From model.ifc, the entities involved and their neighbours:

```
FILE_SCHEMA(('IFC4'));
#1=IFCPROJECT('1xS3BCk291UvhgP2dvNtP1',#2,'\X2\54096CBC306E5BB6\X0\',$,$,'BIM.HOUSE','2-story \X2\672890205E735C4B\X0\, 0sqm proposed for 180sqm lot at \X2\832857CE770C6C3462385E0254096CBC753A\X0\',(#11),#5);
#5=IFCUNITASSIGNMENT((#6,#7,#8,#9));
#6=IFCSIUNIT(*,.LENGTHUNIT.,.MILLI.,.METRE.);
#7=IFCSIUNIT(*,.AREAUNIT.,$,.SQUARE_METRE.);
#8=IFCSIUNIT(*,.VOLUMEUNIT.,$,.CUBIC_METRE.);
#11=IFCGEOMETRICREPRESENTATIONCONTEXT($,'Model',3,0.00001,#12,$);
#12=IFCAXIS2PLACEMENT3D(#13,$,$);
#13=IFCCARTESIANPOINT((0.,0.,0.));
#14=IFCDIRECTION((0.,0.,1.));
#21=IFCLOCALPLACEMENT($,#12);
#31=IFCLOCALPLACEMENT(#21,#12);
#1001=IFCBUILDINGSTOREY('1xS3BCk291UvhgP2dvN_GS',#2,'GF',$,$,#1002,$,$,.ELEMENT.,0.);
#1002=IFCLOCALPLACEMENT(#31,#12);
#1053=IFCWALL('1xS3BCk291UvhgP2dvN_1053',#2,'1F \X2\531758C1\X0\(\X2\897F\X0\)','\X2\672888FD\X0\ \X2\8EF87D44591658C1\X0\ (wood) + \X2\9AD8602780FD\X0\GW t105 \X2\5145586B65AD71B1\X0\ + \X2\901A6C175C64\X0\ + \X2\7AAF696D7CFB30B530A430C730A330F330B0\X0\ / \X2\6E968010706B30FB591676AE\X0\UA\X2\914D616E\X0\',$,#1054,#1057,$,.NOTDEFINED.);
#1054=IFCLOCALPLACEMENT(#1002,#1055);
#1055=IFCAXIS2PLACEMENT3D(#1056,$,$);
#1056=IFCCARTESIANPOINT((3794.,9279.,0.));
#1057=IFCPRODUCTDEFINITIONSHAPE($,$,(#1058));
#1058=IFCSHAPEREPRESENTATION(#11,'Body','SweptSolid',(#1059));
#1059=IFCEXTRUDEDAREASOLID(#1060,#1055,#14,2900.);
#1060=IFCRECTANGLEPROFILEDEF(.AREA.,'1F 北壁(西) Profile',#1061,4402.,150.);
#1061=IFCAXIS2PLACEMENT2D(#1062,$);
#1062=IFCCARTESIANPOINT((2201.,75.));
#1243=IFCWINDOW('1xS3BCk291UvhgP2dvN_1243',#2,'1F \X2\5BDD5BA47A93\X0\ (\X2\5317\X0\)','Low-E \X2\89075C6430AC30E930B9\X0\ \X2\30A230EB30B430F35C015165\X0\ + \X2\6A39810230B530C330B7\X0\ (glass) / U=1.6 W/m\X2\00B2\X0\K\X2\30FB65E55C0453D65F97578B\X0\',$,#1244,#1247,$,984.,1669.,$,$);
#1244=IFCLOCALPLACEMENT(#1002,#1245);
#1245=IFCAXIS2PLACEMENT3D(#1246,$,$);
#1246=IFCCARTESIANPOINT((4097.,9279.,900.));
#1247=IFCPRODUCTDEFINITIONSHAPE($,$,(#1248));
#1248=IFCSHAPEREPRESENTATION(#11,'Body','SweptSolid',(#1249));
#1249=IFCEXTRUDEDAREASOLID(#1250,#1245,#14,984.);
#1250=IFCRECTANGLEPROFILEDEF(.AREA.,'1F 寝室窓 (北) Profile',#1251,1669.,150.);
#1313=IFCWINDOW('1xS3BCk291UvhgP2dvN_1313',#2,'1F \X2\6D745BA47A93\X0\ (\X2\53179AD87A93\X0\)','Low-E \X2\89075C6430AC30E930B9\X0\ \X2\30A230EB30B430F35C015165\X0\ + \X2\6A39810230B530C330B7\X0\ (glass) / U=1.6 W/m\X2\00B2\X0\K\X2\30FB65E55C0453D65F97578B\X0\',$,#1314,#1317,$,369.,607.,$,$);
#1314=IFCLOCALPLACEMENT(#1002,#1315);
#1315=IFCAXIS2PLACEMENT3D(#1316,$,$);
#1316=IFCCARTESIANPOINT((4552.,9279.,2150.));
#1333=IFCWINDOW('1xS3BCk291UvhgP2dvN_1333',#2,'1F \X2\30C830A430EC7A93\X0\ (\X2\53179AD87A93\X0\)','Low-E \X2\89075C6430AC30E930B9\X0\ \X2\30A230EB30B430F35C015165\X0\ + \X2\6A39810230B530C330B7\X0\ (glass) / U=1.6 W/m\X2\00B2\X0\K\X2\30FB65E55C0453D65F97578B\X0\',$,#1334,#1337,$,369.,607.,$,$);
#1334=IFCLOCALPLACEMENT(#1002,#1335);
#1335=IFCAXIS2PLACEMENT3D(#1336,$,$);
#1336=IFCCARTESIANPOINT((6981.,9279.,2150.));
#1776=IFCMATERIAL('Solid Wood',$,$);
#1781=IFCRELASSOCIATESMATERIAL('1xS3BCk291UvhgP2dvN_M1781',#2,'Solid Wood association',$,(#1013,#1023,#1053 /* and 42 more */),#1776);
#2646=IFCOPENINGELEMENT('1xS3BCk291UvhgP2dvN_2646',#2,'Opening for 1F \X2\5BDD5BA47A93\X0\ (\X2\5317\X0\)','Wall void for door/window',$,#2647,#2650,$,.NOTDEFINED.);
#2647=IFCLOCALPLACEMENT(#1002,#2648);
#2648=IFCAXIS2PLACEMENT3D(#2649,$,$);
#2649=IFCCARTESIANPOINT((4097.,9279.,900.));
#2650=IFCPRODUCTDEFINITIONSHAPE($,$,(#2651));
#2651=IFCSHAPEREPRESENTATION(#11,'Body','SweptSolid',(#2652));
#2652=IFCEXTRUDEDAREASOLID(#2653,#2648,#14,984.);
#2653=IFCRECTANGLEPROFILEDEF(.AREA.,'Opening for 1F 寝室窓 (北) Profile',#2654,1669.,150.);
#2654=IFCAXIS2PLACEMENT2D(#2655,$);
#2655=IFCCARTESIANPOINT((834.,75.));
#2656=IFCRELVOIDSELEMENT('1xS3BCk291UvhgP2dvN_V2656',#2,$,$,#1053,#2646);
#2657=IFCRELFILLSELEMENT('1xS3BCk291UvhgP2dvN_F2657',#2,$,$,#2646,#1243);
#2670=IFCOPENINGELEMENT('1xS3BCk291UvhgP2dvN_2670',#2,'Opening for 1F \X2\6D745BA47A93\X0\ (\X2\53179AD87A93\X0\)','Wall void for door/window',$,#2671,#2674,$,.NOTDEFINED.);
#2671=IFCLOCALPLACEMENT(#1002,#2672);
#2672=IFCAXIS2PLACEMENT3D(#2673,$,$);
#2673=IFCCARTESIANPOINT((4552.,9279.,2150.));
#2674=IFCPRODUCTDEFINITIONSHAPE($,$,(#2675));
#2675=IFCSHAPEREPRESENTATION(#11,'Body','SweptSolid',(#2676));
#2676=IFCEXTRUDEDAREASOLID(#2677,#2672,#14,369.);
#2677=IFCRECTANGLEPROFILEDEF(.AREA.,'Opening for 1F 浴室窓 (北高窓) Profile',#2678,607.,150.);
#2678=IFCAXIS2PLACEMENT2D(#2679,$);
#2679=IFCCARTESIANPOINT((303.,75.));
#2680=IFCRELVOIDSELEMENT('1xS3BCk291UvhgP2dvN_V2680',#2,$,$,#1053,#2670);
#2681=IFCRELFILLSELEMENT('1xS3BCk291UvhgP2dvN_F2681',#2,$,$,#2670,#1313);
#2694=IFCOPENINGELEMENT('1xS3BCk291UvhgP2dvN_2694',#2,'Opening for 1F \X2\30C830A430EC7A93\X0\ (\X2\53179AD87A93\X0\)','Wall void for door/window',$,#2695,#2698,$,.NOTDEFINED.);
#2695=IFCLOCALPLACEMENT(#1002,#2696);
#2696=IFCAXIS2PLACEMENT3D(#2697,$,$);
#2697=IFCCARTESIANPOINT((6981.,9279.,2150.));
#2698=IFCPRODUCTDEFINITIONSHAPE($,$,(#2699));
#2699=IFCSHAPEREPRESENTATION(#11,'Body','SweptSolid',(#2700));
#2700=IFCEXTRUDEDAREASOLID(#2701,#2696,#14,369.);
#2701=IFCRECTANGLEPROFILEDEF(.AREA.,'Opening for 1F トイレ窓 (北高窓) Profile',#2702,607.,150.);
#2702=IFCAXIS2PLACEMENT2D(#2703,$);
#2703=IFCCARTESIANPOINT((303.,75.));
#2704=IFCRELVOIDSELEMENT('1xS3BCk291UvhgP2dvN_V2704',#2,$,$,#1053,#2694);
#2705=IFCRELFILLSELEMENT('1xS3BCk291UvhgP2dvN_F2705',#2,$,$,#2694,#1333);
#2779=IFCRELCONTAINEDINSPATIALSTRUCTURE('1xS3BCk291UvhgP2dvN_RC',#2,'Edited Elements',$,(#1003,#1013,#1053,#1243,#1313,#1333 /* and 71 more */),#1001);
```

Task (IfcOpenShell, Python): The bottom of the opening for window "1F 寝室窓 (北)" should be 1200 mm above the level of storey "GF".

```python
import numpy as np
import ifcopenshell
import ifcopenshell.api.geometry
import ifcopenshell.geom
import ifcopenshell.util.element
import ifcopenshell.util.placement
import ifcopenshell.util.shape
import ifcopenshell.util.unit

model = ifcopenshell.open("model.ifc")
unit_scale = ifcopenshell.util.unit.calculate_unit_scale(model)

window = model.by_guid("1xS3BCk291UvhgP2dvN_1243")
opening = window.FillsVoids[0].RelatingOpeningElement
storey = ifcopenshell.util.element.get_container(window, ifc_class="IfcBuildingStorey")
level = ifcopenshell.util.placement.get_local_placement(storey.ObjectPlacement)[2, 3]

# The opening's origin need not be at the sill, so measure its lowest point.
shape = ifcopenshell.geom.create_shape(ifcopenshell.geom.settings(), opening)
bottom = ifcopenshell.util.shape.get_shape_bottom_elevation(shape, shape.geometry) / unit_scale
dz = level + 1200.0 - bottom

shift = np.array([0.0, 0.0, dz])
# The window is not placed relative to its opening, so move both.
for product in (opening, window):
    matrix = ifcopenshell.util.placement.get_local_placement(product.ObjectPlacement)
    matrix[:3, 3] += shift
    ifcopenshell.api.geometry.edit_object_placement(model, product=product, matrix=matrix, is_si=False)

print(f"moved by {dz * unit_scale:+.3f} m")

model.write("model_rev.ifc")
```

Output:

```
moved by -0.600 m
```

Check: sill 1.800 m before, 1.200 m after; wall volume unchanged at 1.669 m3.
